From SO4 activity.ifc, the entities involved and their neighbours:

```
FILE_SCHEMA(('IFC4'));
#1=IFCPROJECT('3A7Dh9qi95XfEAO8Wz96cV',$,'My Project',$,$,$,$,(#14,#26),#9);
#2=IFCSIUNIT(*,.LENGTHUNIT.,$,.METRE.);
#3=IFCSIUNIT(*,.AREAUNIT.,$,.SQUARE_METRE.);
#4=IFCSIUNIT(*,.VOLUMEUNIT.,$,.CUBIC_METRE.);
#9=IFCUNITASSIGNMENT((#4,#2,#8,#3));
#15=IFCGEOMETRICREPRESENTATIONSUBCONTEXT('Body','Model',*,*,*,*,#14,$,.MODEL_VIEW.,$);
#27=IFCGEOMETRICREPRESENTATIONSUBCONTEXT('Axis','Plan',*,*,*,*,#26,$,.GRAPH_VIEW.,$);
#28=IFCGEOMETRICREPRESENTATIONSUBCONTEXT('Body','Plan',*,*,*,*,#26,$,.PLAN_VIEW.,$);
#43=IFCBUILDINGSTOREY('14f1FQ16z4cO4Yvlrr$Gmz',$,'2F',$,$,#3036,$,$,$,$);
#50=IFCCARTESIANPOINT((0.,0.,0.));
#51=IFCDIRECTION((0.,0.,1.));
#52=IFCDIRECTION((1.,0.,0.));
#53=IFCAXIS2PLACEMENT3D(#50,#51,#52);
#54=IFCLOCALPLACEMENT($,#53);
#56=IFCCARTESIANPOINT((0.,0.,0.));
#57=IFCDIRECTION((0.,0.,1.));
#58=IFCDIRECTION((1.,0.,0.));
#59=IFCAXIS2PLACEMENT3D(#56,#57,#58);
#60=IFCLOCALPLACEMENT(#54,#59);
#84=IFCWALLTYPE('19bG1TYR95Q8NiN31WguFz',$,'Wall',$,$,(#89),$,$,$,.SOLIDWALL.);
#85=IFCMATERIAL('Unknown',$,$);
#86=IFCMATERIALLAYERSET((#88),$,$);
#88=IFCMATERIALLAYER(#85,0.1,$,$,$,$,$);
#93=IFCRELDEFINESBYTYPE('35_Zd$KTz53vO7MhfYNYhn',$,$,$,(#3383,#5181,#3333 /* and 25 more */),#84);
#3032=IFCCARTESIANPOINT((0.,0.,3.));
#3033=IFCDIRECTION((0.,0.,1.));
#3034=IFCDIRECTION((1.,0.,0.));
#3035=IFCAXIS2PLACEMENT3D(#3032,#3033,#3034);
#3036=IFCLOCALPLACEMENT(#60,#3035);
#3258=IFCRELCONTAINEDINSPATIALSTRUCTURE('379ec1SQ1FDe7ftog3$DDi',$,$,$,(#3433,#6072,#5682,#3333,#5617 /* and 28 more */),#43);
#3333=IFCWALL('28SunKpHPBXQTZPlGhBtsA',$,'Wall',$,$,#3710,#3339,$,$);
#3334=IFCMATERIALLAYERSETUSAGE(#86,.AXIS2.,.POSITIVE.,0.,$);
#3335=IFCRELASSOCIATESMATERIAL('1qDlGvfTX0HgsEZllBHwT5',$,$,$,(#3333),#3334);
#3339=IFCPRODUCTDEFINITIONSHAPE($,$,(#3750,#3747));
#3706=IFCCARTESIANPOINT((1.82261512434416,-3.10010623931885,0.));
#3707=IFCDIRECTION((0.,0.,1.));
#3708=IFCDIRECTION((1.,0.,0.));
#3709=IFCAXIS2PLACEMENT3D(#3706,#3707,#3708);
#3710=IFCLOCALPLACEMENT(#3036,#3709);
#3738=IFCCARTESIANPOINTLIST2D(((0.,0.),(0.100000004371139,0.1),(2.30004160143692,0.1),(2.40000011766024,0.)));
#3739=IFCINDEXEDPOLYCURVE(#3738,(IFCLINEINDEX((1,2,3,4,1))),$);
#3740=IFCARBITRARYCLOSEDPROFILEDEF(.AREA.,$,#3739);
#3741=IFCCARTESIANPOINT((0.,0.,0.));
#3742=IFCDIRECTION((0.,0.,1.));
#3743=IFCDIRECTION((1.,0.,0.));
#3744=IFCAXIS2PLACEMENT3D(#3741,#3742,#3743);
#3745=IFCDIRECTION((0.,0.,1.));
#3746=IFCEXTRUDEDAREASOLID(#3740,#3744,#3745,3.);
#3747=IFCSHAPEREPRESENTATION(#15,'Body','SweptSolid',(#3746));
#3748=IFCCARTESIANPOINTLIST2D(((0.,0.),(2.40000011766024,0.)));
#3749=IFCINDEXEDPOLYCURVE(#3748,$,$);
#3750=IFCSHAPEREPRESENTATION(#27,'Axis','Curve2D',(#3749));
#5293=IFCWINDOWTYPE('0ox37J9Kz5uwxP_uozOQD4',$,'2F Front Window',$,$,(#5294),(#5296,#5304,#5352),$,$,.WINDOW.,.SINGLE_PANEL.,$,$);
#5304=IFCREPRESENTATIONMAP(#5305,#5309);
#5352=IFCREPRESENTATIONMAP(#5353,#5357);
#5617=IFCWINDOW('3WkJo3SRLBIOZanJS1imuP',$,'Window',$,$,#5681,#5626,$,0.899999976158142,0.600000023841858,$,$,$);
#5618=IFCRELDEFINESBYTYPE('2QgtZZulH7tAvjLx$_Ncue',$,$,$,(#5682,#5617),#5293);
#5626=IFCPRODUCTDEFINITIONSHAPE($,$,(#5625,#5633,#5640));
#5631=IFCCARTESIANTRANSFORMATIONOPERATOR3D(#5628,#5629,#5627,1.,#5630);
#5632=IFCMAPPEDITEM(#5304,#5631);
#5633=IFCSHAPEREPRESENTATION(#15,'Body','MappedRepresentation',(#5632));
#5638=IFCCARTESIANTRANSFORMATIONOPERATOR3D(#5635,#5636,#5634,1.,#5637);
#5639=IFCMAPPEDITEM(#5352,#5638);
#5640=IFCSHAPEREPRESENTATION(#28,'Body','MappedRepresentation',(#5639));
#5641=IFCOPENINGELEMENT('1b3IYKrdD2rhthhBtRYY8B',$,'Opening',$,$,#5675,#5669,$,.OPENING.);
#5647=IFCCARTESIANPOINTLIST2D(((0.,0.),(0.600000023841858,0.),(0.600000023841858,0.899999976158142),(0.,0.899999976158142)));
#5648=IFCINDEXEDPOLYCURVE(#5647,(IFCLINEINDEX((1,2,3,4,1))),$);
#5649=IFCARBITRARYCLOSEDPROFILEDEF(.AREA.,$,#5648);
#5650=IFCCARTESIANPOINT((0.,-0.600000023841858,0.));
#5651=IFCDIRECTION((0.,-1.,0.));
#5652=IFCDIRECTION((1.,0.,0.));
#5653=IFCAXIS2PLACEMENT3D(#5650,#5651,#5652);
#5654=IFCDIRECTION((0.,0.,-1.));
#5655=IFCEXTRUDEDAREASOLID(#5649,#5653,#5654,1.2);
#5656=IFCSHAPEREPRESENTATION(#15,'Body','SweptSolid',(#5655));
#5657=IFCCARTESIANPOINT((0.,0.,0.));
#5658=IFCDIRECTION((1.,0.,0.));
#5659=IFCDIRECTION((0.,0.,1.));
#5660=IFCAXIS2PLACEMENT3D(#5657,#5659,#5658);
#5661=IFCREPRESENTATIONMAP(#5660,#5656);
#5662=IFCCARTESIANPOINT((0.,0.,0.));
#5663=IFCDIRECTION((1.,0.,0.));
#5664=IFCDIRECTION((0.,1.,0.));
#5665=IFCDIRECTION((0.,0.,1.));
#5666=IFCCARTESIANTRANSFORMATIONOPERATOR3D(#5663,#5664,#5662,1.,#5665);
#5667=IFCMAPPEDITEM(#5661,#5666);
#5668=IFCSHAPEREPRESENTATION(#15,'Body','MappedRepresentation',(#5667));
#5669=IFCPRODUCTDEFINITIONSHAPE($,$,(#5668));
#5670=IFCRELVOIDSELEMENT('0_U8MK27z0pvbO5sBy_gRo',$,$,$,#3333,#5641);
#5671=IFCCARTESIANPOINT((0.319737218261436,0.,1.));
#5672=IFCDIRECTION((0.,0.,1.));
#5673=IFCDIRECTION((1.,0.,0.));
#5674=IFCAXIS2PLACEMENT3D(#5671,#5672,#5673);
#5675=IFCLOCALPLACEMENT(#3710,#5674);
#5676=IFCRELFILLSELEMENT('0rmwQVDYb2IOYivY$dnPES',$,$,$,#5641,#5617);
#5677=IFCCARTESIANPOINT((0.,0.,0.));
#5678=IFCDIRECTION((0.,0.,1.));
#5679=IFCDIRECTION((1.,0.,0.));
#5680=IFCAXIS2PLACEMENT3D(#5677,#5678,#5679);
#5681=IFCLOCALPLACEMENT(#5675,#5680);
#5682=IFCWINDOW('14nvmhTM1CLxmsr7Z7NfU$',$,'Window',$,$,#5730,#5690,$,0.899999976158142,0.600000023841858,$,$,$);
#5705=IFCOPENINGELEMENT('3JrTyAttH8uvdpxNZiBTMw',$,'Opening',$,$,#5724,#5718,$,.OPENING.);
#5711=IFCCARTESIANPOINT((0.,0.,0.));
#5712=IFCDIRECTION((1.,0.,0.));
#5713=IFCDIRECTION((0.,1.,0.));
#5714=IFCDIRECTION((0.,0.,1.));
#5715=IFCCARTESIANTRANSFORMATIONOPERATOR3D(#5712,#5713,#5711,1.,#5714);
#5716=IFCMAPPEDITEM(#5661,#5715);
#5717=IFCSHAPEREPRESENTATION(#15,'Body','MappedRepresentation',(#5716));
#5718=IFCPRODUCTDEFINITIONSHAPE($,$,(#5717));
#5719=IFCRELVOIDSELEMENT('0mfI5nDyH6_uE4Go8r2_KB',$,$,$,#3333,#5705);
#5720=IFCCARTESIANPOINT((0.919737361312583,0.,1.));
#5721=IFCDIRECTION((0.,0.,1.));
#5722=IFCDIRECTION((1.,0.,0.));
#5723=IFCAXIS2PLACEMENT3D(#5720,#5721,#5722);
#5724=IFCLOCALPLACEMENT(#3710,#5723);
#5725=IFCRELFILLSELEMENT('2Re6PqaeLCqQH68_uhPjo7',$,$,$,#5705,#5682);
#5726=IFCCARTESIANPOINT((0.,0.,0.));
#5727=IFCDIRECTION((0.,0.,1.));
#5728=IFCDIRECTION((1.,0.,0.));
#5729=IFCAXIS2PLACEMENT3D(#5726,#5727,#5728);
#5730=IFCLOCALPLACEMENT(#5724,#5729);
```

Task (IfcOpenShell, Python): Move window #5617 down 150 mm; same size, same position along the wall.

```python
import numpy as np
import ifcopenshell
import ifcopenshell.api.geometry
import ifcopenshell.util.placement
import ifcopenshell.util.unit

model = ifcopenshell.open("SO4 activity.ifc")
unit_scale = ifcopenshell.util.unit.calculate_unit_scale(model)

window = model.by_guid("3WkJo3SRLBIOZanJS1imuP")
opening = window.FillsVoids[0].RelatingOpeningElement
dz = -0.15 / unit_scale

shift = np.array([0.0, 0.0, dz])
# The window is placed relative to its opening, so it follows when the opening moves.
matrix = ifcopenshell.util.placement.get_local_placement(opening.ObjectPlacement)
matrix[:3, 3] += shift
ifcopenshell.api.geometry.edit_object_placement(
    model, product=opening, matrix=matrix, is_si=False, should_transform_children=True
)

print(f"moved by {dz * unit_scale:+.3f} m")

model.write("SO4 activity_edited.ifc")
```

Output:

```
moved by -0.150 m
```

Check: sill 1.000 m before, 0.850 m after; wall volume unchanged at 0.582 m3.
